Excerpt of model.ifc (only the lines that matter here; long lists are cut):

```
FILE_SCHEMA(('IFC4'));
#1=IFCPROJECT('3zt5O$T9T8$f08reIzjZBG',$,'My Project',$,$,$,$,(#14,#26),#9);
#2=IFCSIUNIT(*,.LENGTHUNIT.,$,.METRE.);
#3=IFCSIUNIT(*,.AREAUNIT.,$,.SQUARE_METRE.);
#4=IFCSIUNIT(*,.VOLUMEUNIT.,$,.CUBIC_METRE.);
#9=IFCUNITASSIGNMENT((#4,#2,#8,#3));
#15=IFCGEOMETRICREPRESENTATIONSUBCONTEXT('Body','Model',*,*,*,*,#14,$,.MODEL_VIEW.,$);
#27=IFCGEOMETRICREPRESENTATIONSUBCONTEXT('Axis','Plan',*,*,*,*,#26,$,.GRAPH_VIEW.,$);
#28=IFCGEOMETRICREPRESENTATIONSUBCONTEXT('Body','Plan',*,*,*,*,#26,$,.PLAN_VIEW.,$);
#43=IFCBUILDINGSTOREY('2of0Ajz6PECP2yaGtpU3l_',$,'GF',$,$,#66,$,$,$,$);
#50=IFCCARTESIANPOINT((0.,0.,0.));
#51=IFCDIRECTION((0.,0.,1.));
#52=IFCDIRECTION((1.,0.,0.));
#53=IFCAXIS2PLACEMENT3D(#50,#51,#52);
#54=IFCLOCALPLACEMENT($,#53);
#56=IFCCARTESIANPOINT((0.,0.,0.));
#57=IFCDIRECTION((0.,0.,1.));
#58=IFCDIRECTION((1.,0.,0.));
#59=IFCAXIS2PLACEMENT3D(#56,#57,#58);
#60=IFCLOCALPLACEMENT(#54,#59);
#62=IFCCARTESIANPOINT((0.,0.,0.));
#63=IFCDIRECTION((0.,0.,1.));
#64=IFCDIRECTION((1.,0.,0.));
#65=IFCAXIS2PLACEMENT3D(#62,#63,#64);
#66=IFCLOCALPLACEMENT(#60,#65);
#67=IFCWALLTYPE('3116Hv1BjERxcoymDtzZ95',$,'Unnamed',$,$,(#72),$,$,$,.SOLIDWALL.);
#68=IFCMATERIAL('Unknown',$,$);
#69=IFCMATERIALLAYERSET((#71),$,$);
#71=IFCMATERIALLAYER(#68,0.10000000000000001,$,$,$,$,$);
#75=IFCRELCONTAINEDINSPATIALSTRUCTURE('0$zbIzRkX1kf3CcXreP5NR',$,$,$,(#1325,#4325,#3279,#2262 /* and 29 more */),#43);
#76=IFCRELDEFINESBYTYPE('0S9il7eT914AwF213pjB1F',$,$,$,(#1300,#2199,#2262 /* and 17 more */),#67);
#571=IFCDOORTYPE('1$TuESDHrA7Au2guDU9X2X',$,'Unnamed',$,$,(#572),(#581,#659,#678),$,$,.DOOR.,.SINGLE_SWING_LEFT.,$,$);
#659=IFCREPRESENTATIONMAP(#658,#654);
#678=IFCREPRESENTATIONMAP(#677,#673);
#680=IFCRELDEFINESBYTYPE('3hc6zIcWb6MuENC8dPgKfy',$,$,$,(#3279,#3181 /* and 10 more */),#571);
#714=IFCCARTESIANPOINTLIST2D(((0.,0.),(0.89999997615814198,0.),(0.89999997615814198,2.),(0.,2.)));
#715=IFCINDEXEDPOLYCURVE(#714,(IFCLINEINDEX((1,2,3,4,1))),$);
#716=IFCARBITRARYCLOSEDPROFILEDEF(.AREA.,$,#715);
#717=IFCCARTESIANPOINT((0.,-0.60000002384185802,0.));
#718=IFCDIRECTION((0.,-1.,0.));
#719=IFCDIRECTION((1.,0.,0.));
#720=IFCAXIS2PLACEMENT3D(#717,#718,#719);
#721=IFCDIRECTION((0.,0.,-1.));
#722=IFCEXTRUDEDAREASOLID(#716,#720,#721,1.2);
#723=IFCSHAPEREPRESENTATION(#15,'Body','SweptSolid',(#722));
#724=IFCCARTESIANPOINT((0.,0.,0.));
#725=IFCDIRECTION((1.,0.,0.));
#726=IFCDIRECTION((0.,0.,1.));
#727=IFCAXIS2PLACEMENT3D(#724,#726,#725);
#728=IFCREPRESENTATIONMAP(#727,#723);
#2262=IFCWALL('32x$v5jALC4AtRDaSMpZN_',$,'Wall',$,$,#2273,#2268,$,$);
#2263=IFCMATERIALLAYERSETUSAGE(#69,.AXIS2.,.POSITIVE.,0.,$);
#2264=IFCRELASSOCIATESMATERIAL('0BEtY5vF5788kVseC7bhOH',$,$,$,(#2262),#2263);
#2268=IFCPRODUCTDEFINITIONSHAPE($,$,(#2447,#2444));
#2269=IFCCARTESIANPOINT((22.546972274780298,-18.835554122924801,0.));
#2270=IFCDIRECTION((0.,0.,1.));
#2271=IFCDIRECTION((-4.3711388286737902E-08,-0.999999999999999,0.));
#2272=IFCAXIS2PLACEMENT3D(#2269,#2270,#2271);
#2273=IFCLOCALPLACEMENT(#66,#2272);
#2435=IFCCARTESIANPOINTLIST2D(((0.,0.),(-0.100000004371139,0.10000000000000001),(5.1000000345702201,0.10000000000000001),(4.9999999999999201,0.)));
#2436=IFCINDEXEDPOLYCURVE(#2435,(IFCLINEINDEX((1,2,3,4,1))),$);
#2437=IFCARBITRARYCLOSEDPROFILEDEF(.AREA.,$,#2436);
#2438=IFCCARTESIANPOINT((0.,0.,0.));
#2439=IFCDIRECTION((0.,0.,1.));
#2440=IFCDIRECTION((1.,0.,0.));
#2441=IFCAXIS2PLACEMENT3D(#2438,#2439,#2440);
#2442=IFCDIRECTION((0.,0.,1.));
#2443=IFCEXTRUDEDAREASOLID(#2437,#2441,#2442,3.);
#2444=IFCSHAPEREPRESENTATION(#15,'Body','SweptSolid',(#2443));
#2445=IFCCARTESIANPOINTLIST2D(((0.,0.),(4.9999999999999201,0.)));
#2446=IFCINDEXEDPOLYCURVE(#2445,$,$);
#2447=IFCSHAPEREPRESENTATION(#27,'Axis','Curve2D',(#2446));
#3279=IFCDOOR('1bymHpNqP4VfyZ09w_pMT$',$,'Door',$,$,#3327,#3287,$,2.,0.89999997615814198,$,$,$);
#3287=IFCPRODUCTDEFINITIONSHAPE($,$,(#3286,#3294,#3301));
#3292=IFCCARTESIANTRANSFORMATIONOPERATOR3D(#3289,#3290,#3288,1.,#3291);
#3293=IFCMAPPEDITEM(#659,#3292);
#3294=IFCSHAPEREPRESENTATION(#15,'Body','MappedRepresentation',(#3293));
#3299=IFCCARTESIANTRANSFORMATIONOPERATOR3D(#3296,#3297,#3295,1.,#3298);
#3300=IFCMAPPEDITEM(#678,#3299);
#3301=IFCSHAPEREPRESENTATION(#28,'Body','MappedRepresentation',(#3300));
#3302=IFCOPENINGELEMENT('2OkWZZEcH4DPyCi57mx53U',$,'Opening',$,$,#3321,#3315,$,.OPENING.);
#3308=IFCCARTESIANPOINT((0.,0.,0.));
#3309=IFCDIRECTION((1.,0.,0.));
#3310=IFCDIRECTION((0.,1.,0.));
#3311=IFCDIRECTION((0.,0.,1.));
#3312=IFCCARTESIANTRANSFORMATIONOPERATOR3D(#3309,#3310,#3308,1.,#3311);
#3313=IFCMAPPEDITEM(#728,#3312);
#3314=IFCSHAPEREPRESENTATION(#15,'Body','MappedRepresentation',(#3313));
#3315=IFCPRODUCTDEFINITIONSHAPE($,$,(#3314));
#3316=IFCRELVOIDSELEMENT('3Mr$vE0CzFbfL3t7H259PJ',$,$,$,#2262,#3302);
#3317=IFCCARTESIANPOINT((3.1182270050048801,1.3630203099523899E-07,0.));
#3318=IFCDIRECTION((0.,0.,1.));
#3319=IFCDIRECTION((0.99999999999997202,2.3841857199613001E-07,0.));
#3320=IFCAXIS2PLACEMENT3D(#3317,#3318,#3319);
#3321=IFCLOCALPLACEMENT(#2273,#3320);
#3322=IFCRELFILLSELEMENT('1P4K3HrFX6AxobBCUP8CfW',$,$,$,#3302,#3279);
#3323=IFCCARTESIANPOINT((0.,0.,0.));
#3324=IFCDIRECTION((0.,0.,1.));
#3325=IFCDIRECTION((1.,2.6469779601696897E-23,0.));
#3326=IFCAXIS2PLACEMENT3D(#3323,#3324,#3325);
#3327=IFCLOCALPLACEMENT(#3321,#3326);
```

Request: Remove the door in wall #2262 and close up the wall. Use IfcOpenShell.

```python
import ifcopenshell
import ifcopenshell.api.feature
import ifcopenshell.api.root
import ifcopenshell.geom
import ifcopenshell.util.shape

model = ifcopenshell.open("model.ifc")
settings = ifcopenshell.geom.settings()


def volume(element):
    """Net volume in cubic metres, openings subtracted."""
    shape = ifcopenshell.geom.create_shape(settings, element)
    return ifcopenshell.util.shape.get_volume(shape.geometry)


door = model.by_guid("1bymHpNqP4VfyZ09w_pMT$")
opening = door.FillsVoids[0].RelatingOpeningElement
wall = opening.VoidsElements[0].RelatingBuildingElement
before = volume(wall)

ifcopenshell.api.root.remove_product(model, product=door)
ifcopenshell.api.feature.remove_feature(model, feature=opening)

after = volume(wall)

print(f"wall volume {before:.3f} -> {after:.3f} m3")

model.write("model_edited.ifc")
```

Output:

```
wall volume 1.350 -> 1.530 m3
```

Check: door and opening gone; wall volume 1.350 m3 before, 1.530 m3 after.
